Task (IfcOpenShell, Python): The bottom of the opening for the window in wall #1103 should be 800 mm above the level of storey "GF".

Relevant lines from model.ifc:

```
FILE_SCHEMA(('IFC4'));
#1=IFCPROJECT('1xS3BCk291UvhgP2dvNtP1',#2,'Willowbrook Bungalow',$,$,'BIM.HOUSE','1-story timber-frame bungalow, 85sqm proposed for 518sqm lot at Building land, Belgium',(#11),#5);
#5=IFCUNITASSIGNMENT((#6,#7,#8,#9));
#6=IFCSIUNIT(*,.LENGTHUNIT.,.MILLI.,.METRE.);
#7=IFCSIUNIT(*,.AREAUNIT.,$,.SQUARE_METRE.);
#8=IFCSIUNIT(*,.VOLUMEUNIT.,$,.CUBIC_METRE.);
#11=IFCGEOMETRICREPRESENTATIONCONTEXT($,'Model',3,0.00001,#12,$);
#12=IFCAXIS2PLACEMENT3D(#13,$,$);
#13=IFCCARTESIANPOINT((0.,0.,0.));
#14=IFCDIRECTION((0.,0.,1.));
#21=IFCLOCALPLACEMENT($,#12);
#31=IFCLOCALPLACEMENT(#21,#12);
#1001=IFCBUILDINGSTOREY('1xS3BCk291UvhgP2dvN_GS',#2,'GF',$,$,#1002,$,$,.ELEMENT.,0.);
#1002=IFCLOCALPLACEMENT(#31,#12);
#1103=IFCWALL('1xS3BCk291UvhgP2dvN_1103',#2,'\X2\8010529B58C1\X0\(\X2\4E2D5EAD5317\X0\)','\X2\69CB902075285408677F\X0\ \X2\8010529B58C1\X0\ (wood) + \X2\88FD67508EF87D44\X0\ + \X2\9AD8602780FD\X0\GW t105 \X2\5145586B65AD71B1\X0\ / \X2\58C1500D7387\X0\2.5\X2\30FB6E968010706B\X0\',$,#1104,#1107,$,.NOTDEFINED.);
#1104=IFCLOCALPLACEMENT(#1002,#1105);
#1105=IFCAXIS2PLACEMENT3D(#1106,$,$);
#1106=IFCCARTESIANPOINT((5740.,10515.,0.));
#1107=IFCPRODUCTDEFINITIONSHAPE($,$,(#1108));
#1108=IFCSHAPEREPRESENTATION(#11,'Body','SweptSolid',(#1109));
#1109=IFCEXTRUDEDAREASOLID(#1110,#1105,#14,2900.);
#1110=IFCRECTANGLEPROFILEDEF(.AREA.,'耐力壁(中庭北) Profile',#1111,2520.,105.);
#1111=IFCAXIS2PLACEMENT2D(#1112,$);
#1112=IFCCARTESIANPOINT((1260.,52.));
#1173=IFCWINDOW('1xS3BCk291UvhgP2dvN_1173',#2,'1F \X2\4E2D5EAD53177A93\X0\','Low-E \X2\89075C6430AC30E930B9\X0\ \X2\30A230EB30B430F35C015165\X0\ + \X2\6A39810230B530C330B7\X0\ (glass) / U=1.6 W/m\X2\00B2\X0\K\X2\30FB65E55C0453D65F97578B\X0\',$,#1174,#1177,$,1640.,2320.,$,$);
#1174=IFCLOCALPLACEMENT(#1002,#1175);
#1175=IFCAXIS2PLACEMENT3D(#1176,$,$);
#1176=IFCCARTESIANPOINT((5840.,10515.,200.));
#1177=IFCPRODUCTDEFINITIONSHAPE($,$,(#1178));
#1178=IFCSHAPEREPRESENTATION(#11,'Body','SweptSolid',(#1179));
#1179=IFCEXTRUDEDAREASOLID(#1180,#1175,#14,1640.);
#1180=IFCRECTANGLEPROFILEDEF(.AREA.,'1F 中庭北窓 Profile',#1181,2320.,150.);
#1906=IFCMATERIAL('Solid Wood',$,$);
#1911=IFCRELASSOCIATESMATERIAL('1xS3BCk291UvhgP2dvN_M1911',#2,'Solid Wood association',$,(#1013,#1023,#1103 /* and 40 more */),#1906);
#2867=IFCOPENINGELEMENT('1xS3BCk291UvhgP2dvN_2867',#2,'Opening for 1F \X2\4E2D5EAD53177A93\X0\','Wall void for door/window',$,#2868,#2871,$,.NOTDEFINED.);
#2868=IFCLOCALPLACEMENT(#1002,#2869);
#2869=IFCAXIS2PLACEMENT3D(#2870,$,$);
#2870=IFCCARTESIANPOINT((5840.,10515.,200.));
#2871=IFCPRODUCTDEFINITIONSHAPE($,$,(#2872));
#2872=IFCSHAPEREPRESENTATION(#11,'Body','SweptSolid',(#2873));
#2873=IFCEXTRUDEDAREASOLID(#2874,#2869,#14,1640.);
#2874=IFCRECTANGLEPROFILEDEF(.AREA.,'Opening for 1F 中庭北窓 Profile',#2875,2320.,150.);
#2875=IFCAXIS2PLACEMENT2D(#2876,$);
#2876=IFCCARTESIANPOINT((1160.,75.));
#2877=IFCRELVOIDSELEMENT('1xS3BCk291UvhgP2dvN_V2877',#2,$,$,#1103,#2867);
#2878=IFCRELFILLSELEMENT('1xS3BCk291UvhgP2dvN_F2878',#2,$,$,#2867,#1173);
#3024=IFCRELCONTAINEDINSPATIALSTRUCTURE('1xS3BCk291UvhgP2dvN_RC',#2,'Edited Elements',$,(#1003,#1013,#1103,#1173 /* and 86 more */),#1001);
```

```python
import numpy as np
import ifcopenshell
import ifcopenshell.api.geometry
import ifcopenshell.geom
import ifcopenshell.util.element
import ifcopenshell.util.placement
import ifcopenshell.util.shape
import ifcopenshell.util.unit

model = ifcopenshell.open("model.ifc")
unit_scale = ifcopenshell.util.unit.calculate_unit_scale(model)

window = model.by_guid("1xS3BCk291UvhgP2dvN_1173")
opening = window.FillsVoids[0].RelatingOpeningElement
storey = ifcopenshell.util.element.get_container(window, ifc_class="IfcBuildingStorey")
level = ifcopenshell.util.placement.get_local_placement(storey.ObjectPlacement)[2, 3]

# The opening's origin need not be at the sill, so measure its lowest point.
shape = ifcopenshell.geom.create_shape(ifcopenshell.geom.settings(), opening)
bottom = ifcopenshell.util.shape.get_shape_bottom_elevation(shape, shape.geometry) / unit_scale
dz = level + 0.8 / unit_scale - bottom

shift = np.array([0.0, 0.0, dz])
# The window is not placed relative to its opening, so move both.
for product in (opening, window):
    matrix = ifcopenshell.util.placement.get_local_placement(product.ObjectPlacement)
    matrix[:3, 3] += shift
    ifcopenshell.api.geometry.edit_object_placement(model, product=product, matrix=matrix, is_si=False)

print(f"moved by {dz * unit_scale:+.3f} m")

model.write("model-out.ifc")
```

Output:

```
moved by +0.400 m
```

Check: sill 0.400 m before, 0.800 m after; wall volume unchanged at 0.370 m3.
